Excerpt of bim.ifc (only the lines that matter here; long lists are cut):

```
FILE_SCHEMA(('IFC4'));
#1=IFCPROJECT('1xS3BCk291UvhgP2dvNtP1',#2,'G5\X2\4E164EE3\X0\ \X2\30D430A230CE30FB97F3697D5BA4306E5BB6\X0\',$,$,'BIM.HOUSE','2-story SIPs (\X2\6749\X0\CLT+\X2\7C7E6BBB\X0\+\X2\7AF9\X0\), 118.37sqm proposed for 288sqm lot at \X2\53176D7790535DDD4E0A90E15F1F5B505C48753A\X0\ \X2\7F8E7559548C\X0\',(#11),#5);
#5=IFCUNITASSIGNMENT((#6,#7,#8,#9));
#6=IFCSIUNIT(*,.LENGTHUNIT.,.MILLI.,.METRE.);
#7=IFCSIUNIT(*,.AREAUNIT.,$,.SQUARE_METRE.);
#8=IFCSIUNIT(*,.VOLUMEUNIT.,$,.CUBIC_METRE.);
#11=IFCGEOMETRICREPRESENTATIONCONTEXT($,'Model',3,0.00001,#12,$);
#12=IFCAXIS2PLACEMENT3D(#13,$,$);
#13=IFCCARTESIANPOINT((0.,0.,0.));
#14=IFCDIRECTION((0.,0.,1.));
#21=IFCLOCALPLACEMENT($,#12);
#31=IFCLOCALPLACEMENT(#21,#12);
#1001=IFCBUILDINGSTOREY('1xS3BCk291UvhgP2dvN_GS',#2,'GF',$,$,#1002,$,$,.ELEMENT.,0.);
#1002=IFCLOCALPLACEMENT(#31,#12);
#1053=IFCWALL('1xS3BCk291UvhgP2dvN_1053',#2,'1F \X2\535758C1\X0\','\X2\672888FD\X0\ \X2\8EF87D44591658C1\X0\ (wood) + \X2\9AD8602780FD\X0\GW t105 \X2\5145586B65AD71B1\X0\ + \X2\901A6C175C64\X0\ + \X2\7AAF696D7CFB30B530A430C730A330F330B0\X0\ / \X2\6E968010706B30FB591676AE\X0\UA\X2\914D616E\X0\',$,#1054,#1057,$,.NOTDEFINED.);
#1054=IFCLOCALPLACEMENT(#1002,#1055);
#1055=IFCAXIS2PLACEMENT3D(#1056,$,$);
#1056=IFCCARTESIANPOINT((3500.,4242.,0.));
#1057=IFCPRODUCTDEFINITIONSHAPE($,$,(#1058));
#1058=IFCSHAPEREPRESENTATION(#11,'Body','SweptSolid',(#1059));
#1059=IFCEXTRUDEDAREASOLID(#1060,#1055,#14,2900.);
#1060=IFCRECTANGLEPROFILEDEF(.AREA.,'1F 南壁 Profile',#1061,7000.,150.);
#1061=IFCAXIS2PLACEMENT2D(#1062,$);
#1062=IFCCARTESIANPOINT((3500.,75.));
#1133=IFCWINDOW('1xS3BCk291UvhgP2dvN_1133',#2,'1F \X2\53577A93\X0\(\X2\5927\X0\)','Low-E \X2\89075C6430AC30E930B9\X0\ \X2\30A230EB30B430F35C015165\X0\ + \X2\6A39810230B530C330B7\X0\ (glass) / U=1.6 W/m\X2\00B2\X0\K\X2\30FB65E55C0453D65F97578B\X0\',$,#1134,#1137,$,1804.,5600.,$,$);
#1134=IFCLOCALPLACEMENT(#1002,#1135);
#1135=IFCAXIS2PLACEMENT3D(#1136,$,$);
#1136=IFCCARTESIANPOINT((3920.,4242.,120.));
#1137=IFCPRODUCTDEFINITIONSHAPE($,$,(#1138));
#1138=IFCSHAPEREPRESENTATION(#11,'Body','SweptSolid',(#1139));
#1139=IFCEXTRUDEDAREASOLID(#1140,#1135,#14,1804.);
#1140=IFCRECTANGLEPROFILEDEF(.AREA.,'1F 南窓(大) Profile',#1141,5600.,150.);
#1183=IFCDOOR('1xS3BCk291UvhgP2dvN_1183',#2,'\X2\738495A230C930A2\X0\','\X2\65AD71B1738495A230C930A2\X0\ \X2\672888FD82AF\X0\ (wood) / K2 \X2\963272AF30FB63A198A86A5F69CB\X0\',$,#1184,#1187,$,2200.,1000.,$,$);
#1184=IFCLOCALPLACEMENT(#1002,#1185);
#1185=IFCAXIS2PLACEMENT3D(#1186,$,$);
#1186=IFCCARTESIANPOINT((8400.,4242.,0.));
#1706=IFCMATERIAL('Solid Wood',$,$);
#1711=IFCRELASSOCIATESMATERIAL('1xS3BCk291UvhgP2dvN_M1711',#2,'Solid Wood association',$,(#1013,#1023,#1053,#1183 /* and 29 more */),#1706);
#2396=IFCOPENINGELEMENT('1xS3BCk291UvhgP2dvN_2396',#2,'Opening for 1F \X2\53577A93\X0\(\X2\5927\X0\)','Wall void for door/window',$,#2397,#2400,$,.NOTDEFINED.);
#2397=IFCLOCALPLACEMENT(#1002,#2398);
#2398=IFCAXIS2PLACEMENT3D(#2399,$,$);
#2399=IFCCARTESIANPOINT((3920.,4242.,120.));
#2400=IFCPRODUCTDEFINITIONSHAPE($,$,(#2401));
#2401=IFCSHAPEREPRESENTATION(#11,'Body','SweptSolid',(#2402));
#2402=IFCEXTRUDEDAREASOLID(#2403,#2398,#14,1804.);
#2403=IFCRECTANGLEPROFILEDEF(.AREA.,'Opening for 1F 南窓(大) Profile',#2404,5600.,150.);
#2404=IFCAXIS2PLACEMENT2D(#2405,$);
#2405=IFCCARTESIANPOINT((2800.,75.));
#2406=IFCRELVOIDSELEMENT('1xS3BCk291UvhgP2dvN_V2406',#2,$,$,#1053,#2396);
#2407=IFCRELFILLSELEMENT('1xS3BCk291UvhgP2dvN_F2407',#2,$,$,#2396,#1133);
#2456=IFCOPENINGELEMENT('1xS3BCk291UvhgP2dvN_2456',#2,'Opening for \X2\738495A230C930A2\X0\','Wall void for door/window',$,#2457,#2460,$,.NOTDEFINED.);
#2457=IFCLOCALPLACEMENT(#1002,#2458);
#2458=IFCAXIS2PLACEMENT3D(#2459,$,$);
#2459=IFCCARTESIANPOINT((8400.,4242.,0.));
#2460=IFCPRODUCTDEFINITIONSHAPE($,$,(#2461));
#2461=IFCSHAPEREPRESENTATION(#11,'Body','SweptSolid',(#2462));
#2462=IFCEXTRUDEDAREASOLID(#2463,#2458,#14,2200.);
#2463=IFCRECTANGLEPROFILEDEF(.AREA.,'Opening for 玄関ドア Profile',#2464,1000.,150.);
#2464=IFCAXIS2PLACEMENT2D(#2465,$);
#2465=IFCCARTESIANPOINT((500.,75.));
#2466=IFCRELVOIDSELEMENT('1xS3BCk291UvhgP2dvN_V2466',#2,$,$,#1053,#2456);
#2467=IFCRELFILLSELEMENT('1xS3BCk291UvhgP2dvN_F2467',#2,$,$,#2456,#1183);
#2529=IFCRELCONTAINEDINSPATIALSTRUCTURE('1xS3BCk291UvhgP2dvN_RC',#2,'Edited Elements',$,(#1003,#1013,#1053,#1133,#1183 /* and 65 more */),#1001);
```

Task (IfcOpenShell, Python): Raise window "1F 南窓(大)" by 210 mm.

```python
import numpy as np
import ifcopenshell
import ifcopenshell.api.geometry
import ifcopenshell.util.placement
import ifcopenshell.util.unit

model = ifcopenshell.open("bim.ifc")
unit_scale = ifcopenshell.util.unit.calculate_unit_scale(model)

window = model.by_guid("1xS3BCk291UvhgP2dvN_1133")
opening = window.FillsVoids[0].RelatingOpeningElement
dz = 210.0

shift = np.array([0.0, 0.0, dz])
# The window is not placed relative to its opening, so move both.
for product in (opening, window):
    matrix = ifcopenshell.util.placement.get_local_placement(product.ObjectPlacement)
    matrix[:3, 3] += shift
    ifcopenshell.api.geometry.edit_object_placement(model, product=product, matrix=matrix, is_si=False)

print(f"moved by {dz * unit_scale:+.3f} m")

model.write("bim_edited.ifc")
```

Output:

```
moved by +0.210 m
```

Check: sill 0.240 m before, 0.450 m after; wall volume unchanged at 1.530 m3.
